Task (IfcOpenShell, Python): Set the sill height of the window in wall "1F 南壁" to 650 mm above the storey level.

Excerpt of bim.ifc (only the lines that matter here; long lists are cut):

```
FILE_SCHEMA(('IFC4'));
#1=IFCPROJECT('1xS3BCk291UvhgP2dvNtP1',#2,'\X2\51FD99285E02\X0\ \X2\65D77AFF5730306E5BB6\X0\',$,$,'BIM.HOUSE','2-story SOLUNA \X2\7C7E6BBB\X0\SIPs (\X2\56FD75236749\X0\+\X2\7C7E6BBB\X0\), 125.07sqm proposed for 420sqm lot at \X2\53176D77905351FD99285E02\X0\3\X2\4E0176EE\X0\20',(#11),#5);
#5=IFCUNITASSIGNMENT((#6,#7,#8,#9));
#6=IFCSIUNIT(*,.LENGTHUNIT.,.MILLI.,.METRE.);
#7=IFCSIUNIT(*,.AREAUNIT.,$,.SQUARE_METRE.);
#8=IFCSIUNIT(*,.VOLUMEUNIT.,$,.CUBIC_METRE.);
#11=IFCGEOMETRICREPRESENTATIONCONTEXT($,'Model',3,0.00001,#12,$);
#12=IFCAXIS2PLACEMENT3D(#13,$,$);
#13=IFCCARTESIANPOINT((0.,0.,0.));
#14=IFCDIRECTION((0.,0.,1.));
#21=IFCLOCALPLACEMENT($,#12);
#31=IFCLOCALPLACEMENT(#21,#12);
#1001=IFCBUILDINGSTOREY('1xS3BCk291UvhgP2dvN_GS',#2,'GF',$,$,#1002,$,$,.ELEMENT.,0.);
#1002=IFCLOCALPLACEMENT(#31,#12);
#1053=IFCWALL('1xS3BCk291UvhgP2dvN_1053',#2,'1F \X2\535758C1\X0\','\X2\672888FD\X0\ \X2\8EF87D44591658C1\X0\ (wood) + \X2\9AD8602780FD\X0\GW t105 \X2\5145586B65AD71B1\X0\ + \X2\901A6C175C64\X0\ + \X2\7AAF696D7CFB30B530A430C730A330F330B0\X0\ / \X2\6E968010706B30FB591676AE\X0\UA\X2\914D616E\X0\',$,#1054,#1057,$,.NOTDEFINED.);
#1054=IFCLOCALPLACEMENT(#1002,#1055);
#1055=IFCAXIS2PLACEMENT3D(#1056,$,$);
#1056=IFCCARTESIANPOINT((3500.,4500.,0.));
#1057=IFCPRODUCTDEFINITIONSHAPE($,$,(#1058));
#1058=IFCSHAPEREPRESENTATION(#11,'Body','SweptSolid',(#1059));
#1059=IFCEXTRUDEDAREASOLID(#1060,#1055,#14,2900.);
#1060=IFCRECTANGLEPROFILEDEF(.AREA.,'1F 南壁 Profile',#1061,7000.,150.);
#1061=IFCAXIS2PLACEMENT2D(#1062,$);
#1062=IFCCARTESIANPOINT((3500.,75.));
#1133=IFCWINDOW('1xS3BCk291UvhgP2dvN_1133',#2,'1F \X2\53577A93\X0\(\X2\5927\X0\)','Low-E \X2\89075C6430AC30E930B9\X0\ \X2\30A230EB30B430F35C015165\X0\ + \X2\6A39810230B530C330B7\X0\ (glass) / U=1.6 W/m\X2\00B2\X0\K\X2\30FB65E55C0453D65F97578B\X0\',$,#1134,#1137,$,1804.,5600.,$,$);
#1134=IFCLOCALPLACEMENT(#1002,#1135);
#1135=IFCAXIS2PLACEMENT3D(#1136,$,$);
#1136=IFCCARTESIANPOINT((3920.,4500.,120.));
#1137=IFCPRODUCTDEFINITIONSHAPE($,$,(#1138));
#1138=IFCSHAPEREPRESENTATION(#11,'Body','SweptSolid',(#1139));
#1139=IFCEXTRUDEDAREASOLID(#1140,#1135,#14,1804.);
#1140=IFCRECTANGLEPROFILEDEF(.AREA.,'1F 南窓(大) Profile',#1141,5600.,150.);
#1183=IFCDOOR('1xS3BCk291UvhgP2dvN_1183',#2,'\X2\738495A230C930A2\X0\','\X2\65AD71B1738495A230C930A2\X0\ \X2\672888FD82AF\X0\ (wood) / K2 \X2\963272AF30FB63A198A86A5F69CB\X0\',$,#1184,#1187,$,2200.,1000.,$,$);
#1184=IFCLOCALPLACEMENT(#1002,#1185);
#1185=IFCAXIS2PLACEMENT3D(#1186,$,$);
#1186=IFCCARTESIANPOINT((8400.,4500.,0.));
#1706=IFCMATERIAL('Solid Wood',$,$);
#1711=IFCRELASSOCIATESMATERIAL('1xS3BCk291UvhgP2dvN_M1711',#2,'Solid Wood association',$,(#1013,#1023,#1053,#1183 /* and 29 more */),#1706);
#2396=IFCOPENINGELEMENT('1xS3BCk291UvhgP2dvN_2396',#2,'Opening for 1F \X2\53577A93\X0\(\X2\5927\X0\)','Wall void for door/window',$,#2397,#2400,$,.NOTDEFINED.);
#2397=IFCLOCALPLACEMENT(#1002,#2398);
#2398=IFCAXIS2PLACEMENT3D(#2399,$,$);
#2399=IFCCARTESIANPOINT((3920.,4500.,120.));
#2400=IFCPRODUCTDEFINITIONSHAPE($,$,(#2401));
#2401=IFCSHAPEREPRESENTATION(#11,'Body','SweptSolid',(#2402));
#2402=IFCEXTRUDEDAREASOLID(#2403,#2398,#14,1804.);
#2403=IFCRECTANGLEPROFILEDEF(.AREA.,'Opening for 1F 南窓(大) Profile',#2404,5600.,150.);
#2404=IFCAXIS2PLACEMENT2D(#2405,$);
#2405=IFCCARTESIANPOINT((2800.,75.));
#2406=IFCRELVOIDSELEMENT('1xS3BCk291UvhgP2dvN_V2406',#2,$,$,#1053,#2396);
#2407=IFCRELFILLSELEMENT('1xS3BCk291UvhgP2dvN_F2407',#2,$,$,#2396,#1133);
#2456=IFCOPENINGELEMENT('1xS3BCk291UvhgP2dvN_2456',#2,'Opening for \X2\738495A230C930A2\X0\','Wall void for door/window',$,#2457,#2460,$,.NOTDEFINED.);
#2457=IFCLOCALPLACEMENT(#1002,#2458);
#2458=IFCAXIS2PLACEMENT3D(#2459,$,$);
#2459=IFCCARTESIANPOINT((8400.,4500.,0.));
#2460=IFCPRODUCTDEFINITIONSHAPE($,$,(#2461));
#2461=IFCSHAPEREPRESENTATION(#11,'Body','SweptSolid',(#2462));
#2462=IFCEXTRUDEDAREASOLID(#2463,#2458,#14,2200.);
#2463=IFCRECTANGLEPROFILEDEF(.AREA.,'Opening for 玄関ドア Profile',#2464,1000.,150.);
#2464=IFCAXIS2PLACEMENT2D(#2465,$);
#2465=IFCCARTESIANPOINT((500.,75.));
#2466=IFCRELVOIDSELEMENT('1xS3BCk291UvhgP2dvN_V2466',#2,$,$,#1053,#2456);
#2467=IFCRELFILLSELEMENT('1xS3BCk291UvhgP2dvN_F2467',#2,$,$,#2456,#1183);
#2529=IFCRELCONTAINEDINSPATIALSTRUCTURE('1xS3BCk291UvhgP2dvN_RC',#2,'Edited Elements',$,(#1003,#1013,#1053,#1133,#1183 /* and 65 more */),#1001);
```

```python
import numpy as np
import ifcopenshell
import ifcopenshell.api.geometry
import ifcopenshell.geom
import ifcopenshell.util.element
import ifcopenshell.util.placement
import ifcopenshell.util.shape
import ifcopenshell.util.unit

model = ifcopenshell.open("bim.ifc")
unit_scale = ifcopenshell.util.unit.calculate_unit_scale(model)

window = model.by_guid("1xS3BCk291UvhgP2dvN_1133")
opening = window.FillsVoids[0].RelatingOpeningElement
storey = ifcopenshell.util.element.get_container(window, ifc_class="IfcBuildingStorey")
level = ifcopenshell.util.placement.get_local_placement(storey.ObjectPlacement)[2, 3]

# The opening's origin need not be at the sill, so measure its lowest point.
shape = ifcopenshell.geom.create_shape(ifcopenshell.geom.settings(), opening)
bottom = ifcopenshell.util.shape.get_shape_bottom_elevation(shape, shape.geometry) / unit_scale
dz = level + 0.65 / unit_scale - bottom

shift = np.array([0.0, 0.0, dz])
# The window is not placed relative to its opening, so move both.
for product in (opening, window):
    matrix = ifcopenshell.util.placement.get_local_placement(product.ObjectPlacement)
    matrix[:3, 3] += shift
    ifcopenshell.api.geometry.edit_object_placement(model, product=product, matrix=matrix, is_si=False)

print(f"moved by {dz * unit_scale:+.3f} m")

model.write("bim_updated.ifc")
```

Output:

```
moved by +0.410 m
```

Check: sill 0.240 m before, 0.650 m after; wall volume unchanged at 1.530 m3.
